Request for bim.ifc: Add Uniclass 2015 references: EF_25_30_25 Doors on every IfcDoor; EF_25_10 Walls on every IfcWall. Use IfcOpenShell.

First a look at what the model holds.

```python
import ifcopenshell

model = ifcopenshell.open("bim.ifc")
print(model.schema)
print("classifications:", [c.Name for c in model.by_type("IfcClassification")])
for ifc_class in ("IfcDoor", "IfcRoof", "IfcStair", "IfcWall", "IfcWindow"):
    print(ifc_class, len(model.by_type(ifc_class)))
```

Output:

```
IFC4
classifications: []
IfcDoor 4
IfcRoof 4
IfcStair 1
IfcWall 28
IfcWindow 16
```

```python
import ifcopenshell
import ifcopenshell.api.classification

model = ifcopenshell.open("bim.ifc")

system = ifcopenshell.api.classification.add_classification(model, classification="Uniclass 2015")

codes = {
    "IfcDoor": ("EF_25_30_25", "Doors"),
    "IfcWall": ("EF_25_10", "Walls"),
}
for ifc_class, (code, name) in codes.items():
    products = model.by_type(ifc_class)
    ifcopenshell.api.classification.add_reference(
        model, products=products, classification=system, identification=code, name=name
    )
    print(code, len(products))

model.write("bim-out.ifc")
```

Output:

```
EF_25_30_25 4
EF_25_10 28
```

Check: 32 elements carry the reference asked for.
